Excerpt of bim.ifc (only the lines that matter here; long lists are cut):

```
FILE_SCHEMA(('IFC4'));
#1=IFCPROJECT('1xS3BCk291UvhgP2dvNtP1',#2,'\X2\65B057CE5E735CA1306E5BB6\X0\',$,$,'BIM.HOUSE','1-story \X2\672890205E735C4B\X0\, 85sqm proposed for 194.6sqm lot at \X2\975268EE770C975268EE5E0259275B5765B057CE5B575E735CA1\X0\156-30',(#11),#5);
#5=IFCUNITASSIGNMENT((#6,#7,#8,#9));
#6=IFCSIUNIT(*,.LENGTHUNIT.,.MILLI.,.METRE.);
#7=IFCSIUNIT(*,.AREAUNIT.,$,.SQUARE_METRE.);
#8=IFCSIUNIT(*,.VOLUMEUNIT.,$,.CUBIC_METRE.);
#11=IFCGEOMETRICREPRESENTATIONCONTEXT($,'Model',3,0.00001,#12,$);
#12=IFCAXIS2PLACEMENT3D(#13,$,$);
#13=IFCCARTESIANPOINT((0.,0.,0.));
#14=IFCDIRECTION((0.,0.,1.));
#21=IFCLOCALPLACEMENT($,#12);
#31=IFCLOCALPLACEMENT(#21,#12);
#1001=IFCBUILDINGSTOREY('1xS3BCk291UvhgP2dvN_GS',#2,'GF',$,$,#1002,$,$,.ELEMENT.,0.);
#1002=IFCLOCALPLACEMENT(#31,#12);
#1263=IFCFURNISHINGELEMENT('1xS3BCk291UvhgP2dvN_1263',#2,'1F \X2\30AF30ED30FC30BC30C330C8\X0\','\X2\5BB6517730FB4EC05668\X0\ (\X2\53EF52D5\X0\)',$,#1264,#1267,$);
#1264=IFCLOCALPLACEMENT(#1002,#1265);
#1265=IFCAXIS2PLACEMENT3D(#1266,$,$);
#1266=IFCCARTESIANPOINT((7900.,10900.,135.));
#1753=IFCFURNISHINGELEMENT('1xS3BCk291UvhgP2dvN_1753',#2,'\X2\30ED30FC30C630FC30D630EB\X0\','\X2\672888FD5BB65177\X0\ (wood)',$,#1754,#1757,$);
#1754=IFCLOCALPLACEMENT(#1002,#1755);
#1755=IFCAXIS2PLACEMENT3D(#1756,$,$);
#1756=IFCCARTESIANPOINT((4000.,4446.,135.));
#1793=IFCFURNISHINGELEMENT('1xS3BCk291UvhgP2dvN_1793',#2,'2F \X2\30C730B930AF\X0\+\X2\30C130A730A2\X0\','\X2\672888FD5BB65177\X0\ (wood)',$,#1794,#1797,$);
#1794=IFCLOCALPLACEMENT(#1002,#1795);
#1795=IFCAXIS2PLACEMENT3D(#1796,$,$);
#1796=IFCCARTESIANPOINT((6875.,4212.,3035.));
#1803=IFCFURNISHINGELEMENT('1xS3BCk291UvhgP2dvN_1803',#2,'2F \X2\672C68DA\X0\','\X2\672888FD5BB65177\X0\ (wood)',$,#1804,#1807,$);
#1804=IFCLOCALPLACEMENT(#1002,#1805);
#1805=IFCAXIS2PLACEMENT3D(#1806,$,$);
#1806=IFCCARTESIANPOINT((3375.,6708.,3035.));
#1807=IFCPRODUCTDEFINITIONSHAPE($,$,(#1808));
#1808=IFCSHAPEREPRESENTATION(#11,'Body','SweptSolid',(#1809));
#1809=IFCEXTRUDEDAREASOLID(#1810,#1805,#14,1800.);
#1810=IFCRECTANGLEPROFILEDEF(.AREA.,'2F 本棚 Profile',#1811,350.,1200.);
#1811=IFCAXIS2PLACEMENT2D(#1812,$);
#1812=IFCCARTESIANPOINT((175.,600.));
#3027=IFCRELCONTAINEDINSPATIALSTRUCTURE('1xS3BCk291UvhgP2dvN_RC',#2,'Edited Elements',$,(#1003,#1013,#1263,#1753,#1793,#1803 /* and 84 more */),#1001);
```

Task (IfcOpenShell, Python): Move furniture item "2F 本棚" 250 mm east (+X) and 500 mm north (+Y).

```python
import ifcopenshell
import ifcopenshell.api.geometry
import ifcopenshell.util.placement

model = ifcopenshell.open("bim.ifc")

item = model.by_guid("1xS3BCk291UvhgP2dvN_1803")
matrix = ifcopenshell.util.placement.get_local_placement(item.ObjectPlacement)
matrix[0, 3] += 250.0
matrix[1, 3] += 500.0
ifcopenshell.api.geometry.edit_object_placement(model, product=item, matrix=matrix, is_si=False)

print(ifcopenshell.util.placement.get_local_placement(item.ObjectPlacement).round(3) + 0.0)

model.write("bim_edited.ifc")
```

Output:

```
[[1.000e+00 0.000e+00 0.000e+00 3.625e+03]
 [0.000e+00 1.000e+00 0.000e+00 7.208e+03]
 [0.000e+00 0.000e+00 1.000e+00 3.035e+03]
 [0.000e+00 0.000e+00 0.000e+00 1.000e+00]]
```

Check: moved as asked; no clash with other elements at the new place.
